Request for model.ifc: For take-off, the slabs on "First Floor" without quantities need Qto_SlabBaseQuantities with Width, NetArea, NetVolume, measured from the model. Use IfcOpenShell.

First a look at what the model holds.

```python
import ifcopenshell
import ifcopenshell.util.element
import ifcopenshell.util.unit

model = ifcopenshell.open("model.ifc")
print(model.schema)
for unit_type in ("LENGTHUNIT", "AREAUNIT", "VOLUMEUNIT"):
    print(unit_type, ifcopenshell.util.unit.calculate_unit_scale(model, unit_type))
storey = next(s for s in model.by_type("IfcBuildingStorey") if s.Name == "First Floor")
slabs = [e for e in ifcopenshell.util.element.get_decomposition(storey) if e.is_a("IfcSlab")]
for e in sorted(slabs, key=lambda e: e.id()):
    print(e.id(), e.is_a(), e.Name, list(ifcopenshell.util.element.get_psets(e, qtos_only=True)), sep=" | ")
```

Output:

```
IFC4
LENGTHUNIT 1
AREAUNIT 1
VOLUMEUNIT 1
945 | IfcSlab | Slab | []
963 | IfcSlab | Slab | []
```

```python
import ifcopenshell
import ifcopenshell.api.pset
import ifcopenshell.geom
import ifcopenshell.util.element
import ifcopenshell.util.shape
import ifcopenshell.util.unit

model = ifcopenshell.open("model.ifc")
unit_scale = ifcopenshell.util.unit.calculate_unit_scale(model)
area_scale = ifcopenshell.util.unit.calculate_unit_scale(model, "AREAUNIT")
volume_scale = ifcopenshell.util.unit.calculate_unit_scale(model, "VOLUMEUNIT")
settings = ifcopenshell.geom.settings()

storey = next(s for s in model.by_type("IfcBuildingStorey") if s.Name == "First Floor")
slabs = [e for e in ifcopenshell.util.element.get_decomposition(storey) if e.is_a("IfcSlab")]

for e in sorted(slabs, key=lambda e: e.id()):
    if ifcopenshell.util.element.get_psets(e, qtos_only=True, should_inherit=False):
        continue
    # Geometry comes back in metres, in the element's own axes.
    shape = ifcopenshell.geom.create_shape(settings, e)
    values = {
        "Width": ifcopenshell.util.shape.get_z(shape.geometry) / unit_scale,
        "NetArea": ifcopenshell.util.shape.get_footprint_area(shape.geometry) / area_scale,
        "NetVolume": ifcopenshell.util.shape.get_volume(shape.geometry) / volume_scale,
    }
    qto = ifcopenshell.api.pset.add_qto(model, product=e, name="Qto_SlabBaseQuantities")
    ifcopenshell.api.pset.edit_qto(model, qto=qto, properties=values)
    print(e.id(), {k: round(v, 3) for k, v in values.items()})

model.write("model_updated.ifc")
```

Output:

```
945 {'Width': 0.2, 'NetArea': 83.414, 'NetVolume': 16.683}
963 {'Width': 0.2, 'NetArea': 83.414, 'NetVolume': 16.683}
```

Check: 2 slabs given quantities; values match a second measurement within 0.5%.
